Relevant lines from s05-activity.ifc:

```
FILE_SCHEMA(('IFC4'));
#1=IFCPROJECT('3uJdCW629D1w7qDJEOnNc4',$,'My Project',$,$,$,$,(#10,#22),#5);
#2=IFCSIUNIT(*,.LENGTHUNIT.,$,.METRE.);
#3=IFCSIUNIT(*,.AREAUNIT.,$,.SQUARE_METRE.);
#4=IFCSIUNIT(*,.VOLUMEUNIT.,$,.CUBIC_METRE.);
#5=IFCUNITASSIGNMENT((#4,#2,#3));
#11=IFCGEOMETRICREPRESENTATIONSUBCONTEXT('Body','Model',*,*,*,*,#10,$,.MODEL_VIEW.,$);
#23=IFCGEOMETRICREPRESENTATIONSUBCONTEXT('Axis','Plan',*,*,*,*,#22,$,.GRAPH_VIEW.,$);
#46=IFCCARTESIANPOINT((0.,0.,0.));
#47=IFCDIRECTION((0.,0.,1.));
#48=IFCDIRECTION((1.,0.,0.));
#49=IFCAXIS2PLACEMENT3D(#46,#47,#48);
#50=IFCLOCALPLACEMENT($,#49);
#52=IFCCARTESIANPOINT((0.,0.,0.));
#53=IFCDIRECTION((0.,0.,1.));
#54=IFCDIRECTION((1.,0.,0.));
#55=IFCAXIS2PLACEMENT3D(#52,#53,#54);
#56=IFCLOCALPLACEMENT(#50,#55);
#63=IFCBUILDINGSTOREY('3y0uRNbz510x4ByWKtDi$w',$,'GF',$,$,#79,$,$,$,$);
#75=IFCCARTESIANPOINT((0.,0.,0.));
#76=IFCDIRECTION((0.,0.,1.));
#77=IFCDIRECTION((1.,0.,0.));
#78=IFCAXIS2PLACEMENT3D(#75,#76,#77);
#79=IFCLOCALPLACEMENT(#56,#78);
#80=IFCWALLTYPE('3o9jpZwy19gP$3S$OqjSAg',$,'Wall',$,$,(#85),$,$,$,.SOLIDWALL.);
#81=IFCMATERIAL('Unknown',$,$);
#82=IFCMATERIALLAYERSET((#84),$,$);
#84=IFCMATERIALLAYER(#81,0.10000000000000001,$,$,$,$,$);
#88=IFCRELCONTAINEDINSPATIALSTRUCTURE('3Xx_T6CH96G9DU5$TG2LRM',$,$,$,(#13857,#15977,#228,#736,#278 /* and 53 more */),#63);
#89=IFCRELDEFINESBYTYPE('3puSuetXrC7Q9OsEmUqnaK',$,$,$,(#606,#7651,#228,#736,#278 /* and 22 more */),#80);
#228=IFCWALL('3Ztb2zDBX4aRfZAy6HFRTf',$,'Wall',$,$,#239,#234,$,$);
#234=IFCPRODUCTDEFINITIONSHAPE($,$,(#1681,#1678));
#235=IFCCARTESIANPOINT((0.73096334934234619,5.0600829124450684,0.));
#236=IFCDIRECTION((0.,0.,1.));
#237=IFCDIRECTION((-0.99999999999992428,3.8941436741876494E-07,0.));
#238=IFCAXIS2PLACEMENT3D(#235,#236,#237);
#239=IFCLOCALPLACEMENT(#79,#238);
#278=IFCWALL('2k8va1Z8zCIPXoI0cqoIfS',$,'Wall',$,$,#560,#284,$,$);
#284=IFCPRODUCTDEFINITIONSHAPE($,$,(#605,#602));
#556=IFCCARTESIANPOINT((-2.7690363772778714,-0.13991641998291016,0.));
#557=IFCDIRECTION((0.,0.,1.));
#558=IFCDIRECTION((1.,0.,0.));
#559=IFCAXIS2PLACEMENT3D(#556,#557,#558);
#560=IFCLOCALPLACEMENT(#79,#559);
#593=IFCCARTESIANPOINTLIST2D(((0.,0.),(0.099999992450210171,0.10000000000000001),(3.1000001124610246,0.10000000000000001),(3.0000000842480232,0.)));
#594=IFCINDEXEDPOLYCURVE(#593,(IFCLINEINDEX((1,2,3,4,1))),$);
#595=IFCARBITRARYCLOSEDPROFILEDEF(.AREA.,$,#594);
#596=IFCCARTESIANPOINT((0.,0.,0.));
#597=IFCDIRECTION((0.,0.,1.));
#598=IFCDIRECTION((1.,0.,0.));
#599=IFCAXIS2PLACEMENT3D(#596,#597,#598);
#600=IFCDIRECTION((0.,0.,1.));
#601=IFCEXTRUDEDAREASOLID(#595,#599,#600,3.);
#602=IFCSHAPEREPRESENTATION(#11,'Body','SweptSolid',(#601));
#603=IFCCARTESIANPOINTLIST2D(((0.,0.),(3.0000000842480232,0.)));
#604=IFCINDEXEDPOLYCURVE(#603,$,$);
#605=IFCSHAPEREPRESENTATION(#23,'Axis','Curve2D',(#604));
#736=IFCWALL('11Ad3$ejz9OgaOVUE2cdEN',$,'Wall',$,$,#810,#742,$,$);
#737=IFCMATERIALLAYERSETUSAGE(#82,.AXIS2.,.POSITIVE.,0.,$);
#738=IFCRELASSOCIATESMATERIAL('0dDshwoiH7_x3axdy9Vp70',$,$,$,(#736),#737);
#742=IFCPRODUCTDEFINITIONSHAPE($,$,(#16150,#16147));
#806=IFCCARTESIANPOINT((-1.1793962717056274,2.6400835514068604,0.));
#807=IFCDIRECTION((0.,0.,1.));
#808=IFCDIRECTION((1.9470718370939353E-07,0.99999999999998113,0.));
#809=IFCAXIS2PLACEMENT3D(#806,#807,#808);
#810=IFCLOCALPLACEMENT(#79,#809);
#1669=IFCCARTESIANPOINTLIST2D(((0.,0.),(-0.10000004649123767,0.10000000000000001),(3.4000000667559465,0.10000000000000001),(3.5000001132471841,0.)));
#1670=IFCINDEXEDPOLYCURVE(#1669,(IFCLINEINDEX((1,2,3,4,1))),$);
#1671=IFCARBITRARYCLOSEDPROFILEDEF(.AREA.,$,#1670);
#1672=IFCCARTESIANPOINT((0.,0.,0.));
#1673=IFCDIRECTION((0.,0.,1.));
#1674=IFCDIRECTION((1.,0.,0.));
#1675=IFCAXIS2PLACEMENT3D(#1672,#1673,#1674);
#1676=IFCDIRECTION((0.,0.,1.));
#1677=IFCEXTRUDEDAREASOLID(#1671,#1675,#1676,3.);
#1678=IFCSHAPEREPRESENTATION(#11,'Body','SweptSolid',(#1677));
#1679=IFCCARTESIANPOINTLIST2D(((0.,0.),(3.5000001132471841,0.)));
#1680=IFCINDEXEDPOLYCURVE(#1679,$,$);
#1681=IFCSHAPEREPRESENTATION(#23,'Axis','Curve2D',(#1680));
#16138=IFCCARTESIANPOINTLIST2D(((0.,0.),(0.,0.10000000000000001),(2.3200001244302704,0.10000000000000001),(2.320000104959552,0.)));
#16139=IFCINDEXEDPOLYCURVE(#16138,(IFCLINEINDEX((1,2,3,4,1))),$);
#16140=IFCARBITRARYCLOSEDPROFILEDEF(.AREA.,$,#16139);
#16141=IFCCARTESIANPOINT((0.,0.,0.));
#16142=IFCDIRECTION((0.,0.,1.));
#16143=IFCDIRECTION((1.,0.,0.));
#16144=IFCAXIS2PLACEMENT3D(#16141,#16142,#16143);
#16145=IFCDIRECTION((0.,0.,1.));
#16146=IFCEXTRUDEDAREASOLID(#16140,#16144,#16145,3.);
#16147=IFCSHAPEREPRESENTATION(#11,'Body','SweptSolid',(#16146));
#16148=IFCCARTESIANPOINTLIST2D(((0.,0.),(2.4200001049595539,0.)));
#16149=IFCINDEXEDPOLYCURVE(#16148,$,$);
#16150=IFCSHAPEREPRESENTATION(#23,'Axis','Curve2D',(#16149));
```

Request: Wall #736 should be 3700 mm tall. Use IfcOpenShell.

```python
import ifcopenshell
import ifcopenshell.geom
import ifcopenshell.util.representation
import ifcopenshell.util.shape
import ifcopenshell.util.unit

model = ifcopenshell.open("s05-activity.ifc")
unit_scale = ifcopenshell.util.unit.calculate_unit_scale(model)
settings = ifcopenshell.geom.settings()


def volume(element):
    """Net volume in cubic metres, openings subtracted."""
    shape = ifcopenshell.geom.create_shape(settings, element)
    return ifcopenshell.util.shape.get_volume(shape.geometry)


wall = model.by_guid("11Ad3$ejz9OgaOVUE2cdEN")
before = volume(wall)

body = ifcopenshell.util.representation.get_representation(wall, "Model", "Body")
solid = body.Items[0]
old_height = solid.Depth
solid.Depth = 3.7 / unit_scale
after = volume(wall)

print(f"height {old_height:g} -> {solid.Depth:g}, volume {before:.3f} -> {after:.3f} m3")

model.write("s05-activity_updated.ifc")
```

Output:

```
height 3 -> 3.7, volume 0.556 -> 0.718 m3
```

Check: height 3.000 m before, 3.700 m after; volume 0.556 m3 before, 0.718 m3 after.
